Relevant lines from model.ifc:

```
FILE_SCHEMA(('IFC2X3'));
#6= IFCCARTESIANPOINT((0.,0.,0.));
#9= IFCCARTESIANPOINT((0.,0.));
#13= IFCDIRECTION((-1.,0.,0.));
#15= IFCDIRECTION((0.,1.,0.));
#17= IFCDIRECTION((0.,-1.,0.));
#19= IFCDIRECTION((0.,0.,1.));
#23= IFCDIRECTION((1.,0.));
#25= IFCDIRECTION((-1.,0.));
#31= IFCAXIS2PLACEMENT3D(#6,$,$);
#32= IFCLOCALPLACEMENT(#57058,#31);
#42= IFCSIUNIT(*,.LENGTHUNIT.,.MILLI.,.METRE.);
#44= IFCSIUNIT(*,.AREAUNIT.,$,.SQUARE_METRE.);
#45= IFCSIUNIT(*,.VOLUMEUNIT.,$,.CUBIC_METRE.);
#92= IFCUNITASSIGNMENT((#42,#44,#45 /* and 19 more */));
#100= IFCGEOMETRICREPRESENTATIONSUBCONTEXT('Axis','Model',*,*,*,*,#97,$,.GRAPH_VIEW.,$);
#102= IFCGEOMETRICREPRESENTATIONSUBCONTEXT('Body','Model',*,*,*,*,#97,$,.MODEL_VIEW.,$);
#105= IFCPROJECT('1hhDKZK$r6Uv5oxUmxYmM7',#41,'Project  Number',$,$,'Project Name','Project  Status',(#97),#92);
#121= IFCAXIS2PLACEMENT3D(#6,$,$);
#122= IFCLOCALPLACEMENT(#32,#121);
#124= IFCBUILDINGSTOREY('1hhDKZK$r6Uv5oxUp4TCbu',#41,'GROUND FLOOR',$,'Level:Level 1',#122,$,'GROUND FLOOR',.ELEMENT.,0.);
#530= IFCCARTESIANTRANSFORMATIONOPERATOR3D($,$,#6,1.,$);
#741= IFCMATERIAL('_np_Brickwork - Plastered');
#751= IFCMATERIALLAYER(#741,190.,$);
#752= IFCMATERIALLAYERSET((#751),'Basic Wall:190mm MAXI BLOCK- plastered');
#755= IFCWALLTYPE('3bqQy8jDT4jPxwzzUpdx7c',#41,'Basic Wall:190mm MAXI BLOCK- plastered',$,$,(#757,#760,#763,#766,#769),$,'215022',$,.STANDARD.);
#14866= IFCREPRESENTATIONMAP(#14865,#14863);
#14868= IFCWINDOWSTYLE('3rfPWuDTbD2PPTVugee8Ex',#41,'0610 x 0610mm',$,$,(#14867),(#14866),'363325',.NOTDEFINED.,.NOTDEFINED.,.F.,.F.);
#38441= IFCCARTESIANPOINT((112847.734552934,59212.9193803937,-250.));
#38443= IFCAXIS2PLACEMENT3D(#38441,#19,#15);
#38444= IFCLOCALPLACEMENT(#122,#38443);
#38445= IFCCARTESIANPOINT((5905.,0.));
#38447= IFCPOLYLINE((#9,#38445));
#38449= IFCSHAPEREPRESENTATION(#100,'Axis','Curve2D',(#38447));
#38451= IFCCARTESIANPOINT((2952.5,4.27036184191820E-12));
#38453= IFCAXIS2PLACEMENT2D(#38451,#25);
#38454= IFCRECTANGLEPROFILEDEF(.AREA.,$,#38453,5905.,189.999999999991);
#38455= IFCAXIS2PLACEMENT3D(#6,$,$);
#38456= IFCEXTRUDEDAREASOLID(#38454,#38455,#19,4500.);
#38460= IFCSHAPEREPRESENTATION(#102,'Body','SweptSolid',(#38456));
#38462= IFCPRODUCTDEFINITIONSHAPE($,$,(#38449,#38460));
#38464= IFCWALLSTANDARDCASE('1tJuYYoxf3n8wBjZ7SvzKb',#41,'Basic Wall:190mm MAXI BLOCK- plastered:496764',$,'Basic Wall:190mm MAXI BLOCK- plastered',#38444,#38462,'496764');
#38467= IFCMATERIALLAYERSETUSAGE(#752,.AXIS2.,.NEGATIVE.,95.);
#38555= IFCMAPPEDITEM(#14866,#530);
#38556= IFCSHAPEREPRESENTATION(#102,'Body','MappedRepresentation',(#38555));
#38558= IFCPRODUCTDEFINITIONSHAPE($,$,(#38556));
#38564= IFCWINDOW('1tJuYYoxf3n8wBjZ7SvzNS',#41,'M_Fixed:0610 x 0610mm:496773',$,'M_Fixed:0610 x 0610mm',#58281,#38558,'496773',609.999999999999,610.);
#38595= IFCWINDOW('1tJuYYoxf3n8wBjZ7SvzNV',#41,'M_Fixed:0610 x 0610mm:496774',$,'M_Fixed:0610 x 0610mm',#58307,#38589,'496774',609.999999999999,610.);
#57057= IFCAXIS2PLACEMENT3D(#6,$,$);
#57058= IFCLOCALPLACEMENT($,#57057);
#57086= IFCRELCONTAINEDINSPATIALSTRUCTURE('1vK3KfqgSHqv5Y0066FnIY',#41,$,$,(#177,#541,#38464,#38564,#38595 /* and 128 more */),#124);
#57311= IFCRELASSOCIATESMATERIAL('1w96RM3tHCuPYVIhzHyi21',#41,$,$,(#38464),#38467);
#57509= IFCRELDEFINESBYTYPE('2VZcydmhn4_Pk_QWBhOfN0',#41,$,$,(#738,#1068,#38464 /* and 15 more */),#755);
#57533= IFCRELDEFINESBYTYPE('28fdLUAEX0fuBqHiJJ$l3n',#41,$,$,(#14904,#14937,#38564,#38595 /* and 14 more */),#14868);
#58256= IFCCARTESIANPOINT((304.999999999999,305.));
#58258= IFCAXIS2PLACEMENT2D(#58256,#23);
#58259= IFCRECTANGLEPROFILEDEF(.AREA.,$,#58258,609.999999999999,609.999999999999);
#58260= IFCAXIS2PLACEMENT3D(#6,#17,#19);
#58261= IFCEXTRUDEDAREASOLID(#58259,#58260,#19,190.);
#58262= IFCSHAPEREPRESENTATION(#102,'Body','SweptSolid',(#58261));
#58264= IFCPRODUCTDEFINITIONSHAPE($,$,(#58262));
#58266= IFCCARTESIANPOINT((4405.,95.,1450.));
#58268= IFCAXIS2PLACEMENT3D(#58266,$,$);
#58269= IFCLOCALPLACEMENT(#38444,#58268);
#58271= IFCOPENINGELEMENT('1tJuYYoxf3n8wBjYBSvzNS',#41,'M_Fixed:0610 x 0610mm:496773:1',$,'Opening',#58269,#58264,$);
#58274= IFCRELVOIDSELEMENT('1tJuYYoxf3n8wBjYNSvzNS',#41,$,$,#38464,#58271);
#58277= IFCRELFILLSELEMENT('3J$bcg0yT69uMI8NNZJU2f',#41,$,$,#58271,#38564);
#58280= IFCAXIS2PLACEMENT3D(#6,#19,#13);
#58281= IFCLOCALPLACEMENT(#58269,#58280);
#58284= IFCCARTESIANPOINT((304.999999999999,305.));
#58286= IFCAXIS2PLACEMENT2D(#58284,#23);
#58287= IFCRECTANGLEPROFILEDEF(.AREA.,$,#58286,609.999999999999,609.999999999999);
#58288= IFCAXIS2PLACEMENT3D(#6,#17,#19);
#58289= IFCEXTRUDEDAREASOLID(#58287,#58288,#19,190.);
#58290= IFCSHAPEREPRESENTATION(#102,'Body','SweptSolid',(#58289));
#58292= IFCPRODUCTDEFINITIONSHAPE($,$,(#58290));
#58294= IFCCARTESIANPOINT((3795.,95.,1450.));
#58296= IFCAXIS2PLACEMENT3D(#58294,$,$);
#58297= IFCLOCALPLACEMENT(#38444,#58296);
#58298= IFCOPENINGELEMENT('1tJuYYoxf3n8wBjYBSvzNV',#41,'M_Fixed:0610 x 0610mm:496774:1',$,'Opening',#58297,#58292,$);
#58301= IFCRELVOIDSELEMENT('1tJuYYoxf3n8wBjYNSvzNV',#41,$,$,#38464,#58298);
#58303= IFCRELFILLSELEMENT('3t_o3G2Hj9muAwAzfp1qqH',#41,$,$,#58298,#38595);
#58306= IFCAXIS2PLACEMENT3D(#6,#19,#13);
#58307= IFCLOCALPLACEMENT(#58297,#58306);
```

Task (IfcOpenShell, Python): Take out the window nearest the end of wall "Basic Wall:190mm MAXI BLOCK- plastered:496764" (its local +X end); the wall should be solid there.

```python
import ifcopenshell
import ifcopenshell.api.feature
import ifcopenshell.api.root
import ifcopenshell.geom
import ifcopenshell.util.shape

model = ifcopenshell.open("model.ifc")
settings = ifcopenshell.geom.settings()


def volume(element):
    """Net volume in cubic metres, openings subtracted."""
    shape = ifcopenshell.geom.create_shape(settings, element)
    return ifcopenshell.util.shape.get_volume(shape.geometry)


window = model.by_guid("1tJuYYoxf3n8wBjZ7SvzNS")
opening = window.FillsVoids[0].RelatingOpeningElement
wall = opening.VoidsElements[0].RelatingBuildingElement
before = volume(wall)

ifcopenshell.api.root.remove_product(model, product=window)
ifcopenshell.api.feature.remove_feature(model, feature=opening)

after = volume(wall)

print(f"wall volume {before:.3f} -> {after:.3f} m3")

model.write("model-out.ifc")
```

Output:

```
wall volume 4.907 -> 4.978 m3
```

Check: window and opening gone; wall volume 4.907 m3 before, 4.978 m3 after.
